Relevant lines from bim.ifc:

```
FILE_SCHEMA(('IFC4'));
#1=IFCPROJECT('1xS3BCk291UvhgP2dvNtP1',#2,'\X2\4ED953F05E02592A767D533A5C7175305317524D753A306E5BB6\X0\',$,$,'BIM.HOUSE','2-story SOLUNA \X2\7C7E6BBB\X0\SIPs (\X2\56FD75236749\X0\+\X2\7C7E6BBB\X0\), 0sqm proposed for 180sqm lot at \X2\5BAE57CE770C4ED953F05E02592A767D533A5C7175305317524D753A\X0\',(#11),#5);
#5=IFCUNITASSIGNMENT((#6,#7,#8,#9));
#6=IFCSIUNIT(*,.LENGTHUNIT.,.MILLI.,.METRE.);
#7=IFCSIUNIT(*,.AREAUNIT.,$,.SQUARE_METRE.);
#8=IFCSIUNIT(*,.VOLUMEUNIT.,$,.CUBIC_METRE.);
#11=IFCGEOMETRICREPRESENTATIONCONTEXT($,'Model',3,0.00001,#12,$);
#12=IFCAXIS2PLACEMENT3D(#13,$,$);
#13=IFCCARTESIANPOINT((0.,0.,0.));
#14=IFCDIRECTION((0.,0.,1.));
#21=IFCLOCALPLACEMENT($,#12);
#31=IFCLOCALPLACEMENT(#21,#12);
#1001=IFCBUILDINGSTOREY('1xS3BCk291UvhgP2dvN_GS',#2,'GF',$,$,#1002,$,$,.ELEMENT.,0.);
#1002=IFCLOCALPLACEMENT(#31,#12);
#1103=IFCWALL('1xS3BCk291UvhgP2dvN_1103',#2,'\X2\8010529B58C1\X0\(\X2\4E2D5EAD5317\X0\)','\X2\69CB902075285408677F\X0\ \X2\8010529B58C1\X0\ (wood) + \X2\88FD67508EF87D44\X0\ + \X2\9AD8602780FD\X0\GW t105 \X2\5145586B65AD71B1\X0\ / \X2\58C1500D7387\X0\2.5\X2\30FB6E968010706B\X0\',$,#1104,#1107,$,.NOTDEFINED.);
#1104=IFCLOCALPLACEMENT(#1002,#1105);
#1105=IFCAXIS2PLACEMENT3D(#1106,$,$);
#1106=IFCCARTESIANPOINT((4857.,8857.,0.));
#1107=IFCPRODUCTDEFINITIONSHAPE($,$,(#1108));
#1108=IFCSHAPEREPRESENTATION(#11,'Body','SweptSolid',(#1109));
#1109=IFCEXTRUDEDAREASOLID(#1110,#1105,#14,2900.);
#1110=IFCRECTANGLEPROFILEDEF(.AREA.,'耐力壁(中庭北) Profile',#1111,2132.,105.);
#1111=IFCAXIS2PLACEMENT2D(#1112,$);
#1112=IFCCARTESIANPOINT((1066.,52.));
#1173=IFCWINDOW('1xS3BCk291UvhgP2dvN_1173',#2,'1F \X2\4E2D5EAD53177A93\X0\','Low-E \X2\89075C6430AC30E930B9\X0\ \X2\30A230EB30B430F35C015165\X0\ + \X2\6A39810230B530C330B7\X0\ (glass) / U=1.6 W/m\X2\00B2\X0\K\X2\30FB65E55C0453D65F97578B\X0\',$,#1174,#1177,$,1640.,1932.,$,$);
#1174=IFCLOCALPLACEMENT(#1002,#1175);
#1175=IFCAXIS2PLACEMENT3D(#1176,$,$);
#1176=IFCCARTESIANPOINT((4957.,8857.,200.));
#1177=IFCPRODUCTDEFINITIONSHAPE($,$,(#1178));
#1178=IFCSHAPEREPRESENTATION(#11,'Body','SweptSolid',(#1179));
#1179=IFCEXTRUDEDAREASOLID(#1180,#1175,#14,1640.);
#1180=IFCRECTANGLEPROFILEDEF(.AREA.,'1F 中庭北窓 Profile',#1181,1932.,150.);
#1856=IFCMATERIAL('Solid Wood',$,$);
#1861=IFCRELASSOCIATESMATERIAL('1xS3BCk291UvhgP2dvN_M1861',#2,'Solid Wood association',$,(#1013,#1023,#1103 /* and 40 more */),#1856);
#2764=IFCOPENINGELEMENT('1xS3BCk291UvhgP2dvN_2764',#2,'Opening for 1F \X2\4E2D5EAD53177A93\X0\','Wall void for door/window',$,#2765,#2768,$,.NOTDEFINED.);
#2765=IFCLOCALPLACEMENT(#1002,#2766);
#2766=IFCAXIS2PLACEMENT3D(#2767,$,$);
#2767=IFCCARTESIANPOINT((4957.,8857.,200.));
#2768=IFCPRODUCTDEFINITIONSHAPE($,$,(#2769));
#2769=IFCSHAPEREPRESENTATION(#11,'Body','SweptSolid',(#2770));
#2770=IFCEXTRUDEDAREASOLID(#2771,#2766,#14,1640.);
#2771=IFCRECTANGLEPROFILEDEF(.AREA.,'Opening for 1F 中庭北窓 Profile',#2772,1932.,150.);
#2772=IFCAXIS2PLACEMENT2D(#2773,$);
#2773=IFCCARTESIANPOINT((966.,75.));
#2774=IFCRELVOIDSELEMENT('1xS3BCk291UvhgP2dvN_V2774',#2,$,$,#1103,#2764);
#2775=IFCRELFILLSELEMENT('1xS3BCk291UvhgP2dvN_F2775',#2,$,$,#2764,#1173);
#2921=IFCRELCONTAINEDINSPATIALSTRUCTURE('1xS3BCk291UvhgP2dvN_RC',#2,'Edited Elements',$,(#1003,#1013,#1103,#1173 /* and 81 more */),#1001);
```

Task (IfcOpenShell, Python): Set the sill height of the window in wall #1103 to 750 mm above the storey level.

```python
import numpy as np
import ifcopenshell
import ifcopenshell.api.geometry
import ifcopenshell.geom
import ifcopenshell.util.element
import ifcopenshell.util.placement
import ifcopenshell.util.shape
import ifcopenshell.util.unit

model = ifcopenshell.open("bim.ifc")
unit_scale = ifcopenshell.util.unit.calculate_unit_scale(model)

window = model.by_id(1173)
opening = window.FillsVoids[0].RelatingOpeningElement
storey = ifcopenshell.util.element.get_container(window, ifc_class="IfcBuildingStorey")
level = ifcopenshell.util.placement.get_local_placement(storey.ObjectPlacement)[2, 3]

# The opening's origin need not be at the sill, so measure its lowest point.
shape = ifcopenshell.geom.create_shape(ifcopenshell.geom.settings(), opening)
bottom = ifcopenshell.util.shape.get_shape_bottom_elevation(shape, shape.geometry) / unit_scale
dz = level + 0.75 / unit_scale - bottom

shift = np.array([0.0, 0.0, dz])
# The window is not placed relative to its opening, so move both.
for product in (opening, window):
    matrix = ifcopenshell.util.placement.get_local_placement(product.ObjectPlacement)
    matrix[:3, 3] += shift
    ifcopenshell.api.geometry.edit_object_placement(model, product=product, matrix=matrix, is_si=False)

print(f"moved by {dz * unit_scale:+.3f} m")

model.write("bim_rev.ifc")
```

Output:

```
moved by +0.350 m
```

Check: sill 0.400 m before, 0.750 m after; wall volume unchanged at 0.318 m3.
